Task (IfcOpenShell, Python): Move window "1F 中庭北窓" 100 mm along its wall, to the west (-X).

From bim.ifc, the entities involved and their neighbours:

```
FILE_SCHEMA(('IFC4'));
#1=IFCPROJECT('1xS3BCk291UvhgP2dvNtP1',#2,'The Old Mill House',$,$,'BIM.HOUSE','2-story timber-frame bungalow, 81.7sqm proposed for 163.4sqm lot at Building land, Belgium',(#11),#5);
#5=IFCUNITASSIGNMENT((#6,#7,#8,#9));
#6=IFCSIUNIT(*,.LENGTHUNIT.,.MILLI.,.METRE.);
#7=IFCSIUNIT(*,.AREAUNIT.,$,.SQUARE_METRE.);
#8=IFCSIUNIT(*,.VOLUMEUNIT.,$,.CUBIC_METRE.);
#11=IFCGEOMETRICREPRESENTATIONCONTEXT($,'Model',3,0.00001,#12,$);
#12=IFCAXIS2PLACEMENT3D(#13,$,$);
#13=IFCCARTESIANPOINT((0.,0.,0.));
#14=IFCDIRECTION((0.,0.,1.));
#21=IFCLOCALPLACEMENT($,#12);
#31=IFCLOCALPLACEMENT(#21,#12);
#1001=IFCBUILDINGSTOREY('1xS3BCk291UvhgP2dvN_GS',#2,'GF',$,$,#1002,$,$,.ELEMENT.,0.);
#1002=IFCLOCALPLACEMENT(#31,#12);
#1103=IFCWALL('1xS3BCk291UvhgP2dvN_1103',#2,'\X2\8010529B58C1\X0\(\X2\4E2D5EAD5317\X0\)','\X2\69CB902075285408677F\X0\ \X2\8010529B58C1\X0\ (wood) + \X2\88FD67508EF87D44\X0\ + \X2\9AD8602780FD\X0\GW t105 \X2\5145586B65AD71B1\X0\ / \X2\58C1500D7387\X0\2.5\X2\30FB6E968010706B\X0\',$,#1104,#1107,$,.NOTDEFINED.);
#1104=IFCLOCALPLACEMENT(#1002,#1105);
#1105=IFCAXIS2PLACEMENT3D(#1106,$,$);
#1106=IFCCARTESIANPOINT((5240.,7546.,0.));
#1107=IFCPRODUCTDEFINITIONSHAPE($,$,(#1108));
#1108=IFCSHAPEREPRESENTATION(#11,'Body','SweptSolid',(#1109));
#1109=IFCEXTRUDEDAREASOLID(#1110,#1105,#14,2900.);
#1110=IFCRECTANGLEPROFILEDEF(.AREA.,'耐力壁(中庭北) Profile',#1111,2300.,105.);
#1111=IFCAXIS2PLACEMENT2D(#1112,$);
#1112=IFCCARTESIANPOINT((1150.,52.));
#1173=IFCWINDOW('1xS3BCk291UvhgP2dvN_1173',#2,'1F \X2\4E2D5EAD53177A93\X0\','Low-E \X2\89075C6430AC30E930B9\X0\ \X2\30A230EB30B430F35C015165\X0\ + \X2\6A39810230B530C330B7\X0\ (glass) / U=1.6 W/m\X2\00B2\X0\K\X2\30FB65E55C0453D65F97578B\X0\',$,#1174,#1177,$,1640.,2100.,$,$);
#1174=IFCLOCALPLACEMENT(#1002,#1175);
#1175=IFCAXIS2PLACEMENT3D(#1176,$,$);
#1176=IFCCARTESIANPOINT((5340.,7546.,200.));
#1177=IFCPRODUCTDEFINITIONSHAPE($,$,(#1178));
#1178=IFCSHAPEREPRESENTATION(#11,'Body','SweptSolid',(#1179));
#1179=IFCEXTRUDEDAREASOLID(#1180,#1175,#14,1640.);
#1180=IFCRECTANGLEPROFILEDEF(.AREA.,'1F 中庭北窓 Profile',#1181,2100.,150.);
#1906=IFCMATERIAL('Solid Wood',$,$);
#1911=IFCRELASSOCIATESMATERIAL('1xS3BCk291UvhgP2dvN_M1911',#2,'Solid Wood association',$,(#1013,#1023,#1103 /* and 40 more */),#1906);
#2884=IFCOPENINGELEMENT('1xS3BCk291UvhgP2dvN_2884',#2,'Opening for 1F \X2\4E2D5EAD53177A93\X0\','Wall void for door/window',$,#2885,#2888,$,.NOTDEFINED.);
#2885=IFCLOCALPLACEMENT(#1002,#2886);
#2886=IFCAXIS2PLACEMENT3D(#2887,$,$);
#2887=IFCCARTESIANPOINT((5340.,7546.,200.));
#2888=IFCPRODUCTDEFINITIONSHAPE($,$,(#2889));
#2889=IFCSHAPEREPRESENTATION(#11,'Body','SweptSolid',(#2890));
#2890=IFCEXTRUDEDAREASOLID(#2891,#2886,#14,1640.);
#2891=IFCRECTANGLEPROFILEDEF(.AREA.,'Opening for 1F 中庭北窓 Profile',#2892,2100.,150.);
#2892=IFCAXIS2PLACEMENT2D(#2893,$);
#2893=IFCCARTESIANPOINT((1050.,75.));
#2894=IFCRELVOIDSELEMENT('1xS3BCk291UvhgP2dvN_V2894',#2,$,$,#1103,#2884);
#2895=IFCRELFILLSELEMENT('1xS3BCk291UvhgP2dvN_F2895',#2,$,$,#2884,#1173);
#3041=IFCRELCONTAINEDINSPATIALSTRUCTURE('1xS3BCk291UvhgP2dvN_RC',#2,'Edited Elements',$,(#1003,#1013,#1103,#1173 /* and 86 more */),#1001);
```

```python
import ifcopenshell
import ifcopenshell.api.geometry
import ifcopenshell.util.placement
import ifcopenshell.util.unit

model = ifcopenshell.open("bim.ifc")
unit_scale = ifcopenshell.util.unit.calculate_unit_scale(model)

window = model.by_id(1173)
opening = window.FillsVoids[0].RelatingOpeningElement
wall = opening.VoidsElements[0].RelatingBuildingElement

wall_matrix = ifcopenshell.util.placement.get_local_placement(wall.ObjectPlacement)
shift = wall_matrix[:3, 0] * -0.1 / unit_scale
before = ifcopenshell.util.placement.get_local_placement(window.ObjectPlacement)[:3, 3].copy()

# The window is not placed relative to its opening, so move both.
for product in (opening, window):
    matrix = ifcopenshell.util.placement.get_local_placement(product.ObjectPlacement)
    matrix[:3, 3] += shift
    ifcopenshell.api.geometry.edit_object_placement(model, product=product, matrix=matrix, is_si=False)

after = ifcopenshell.util.placement.get_local_placement(window.ObjectPlacement)[:3, 3]
print("window moved by", (after - before).round(3) + 0.0)

model.write("bim-out.ifc")
```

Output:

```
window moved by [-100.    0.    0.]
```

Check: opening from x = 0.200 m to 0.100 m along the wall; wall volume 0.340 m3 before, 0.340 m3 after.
